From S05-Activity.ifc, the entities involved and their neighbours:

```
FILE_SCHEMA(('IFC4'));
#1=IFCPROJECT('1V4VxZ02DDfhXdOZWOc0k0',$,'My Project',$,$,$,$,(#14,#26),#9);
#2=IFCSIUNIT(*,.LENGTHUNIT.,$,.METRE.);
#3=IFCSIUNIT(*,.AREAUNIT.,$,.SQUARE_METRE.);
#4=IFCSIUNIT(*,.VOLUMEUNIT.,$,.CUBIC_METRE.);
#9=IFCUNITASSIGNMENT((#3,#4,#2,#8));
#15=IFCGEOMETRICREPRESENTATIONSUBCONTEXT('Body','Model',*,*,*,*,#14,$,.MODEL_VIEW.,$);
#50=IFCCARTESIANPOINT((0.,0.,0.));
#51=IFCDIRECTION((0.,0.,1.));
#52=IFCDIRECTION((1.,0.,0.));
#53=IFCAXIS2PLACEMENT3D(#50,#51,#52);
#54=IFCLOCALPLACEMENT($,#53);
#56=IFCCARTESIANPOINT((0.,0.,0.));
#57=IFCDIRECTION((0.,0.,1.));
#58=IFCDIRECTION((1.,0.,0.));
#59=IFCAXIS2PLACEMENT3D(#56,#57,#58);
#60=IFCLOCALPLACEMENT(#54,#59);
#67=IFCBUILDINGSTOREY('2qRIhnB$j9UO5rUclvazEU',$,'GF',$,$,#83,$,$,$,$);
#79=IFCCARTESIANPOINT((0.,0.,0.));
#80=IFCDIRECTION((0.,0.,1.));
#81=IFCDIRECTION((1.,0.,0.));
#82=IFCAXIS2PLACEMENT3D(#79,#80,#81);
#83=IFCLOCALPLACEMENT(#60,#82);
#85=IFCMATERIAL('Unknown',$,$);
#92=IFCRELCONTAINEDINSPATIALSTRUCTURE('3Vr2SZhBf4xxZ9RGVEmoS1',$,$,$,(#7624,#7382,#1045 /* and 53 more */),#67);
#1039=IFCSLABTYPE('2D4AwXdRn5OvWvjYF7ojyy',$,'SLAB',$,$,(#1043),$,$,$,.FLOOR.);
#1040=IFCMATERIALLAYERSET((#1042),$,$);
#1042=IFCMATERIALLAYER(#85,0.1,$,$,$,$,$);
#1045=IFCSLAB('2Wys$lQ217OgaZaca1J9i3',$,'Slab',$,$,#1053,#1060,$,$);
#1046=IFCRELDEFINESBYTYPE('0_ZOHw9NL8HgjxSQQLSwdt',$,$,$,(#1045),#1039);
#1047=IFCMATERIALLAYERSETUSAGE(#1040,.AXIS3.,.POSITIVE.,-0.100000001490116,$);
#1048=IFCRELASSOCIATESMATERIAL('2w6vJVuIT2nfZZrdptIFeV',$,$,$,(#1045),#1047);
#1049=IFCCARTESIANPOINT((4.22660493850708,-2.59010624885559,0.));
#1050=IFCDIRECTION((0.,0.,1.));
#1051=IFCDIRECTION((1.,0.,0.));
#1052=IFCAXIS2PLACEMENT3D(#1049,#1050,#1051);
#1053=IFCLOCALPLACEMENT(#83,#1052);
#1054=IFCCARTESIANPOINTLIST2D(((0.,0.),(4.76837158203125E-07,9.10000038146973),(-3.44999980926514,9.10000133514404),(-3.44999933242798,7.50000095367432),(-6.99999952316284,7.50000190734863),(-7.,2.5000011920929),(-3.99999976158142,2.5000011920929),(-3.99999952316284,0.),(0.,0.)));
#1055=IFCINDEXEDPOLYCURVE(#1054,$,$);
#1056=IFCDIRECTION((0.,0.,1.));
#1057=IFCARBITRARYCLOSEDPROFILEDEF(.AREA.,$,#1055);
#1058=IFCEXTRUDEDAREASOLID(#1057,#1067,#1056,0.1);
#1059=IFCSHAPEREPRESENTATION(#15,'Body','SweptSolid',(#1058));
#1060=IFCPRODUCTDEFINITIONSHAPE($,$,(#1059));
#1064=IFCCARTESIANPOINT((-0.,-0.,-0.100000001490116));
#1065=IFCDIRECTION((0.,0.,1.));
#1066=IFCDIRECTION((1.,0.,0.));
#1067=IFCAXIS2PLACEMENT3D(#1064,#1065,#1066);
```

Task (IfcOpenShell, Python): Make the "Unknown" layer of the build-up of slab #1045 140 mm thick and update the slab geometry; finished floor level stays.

```python
import ifcopenshell
import ifcopenshell.util.element
import ifcopenshell.util.representation
import ifcopenshell.util.unit

model = ifcopenshell.open("S05-Activity.ifc")
unit_scale = ifcopenshell.util.unit.calculate_unit_scale(model)

layer_set = model.by_id(1040)
layer = next(l for l in layer_set.MaterialLayers if l.Material and l.Material.Name == "Unknown")
change = 0.14 / unit_scale - layer.LayerThickness
layer.LayerThickness += change

# Geometry does not follow the layer set by itself.
slabs = [e for e in ifcopenshell.util.element.get_elements_by_material(model, layer_set) if e.is_a("IfcSlab")]
for slab in sorted(slabs, key=lambda e: e.id()):
    body = ifcopenshell.util.representation.get_representation(slab, "Model", "Body")
    solid = body.Items[0]
    old_depth = solid.Depth
    solid.Depth += change
    # Extruded upwards: lower the start of the extrusion so the top stays.
    x, y, z = solid.Position.Location.Coordinates
    solid.Position.Location = model.createIfcCartesianPoint((x, y, z - change))
    print(slab.id(), f"{old_depth:g} -> {solid.Depth:g}")

# The layers are counted up from the underside, which has moved.
for usage in {ifcopenshell.util.element.get_material(slab) for slab in slabs}:
    usage.OffsetFromReferenceLine -= change

model.write("S05-Activity_edited.ifc")
```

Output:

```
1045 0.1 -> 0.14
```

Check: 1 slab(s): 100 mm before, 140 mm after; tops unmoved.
